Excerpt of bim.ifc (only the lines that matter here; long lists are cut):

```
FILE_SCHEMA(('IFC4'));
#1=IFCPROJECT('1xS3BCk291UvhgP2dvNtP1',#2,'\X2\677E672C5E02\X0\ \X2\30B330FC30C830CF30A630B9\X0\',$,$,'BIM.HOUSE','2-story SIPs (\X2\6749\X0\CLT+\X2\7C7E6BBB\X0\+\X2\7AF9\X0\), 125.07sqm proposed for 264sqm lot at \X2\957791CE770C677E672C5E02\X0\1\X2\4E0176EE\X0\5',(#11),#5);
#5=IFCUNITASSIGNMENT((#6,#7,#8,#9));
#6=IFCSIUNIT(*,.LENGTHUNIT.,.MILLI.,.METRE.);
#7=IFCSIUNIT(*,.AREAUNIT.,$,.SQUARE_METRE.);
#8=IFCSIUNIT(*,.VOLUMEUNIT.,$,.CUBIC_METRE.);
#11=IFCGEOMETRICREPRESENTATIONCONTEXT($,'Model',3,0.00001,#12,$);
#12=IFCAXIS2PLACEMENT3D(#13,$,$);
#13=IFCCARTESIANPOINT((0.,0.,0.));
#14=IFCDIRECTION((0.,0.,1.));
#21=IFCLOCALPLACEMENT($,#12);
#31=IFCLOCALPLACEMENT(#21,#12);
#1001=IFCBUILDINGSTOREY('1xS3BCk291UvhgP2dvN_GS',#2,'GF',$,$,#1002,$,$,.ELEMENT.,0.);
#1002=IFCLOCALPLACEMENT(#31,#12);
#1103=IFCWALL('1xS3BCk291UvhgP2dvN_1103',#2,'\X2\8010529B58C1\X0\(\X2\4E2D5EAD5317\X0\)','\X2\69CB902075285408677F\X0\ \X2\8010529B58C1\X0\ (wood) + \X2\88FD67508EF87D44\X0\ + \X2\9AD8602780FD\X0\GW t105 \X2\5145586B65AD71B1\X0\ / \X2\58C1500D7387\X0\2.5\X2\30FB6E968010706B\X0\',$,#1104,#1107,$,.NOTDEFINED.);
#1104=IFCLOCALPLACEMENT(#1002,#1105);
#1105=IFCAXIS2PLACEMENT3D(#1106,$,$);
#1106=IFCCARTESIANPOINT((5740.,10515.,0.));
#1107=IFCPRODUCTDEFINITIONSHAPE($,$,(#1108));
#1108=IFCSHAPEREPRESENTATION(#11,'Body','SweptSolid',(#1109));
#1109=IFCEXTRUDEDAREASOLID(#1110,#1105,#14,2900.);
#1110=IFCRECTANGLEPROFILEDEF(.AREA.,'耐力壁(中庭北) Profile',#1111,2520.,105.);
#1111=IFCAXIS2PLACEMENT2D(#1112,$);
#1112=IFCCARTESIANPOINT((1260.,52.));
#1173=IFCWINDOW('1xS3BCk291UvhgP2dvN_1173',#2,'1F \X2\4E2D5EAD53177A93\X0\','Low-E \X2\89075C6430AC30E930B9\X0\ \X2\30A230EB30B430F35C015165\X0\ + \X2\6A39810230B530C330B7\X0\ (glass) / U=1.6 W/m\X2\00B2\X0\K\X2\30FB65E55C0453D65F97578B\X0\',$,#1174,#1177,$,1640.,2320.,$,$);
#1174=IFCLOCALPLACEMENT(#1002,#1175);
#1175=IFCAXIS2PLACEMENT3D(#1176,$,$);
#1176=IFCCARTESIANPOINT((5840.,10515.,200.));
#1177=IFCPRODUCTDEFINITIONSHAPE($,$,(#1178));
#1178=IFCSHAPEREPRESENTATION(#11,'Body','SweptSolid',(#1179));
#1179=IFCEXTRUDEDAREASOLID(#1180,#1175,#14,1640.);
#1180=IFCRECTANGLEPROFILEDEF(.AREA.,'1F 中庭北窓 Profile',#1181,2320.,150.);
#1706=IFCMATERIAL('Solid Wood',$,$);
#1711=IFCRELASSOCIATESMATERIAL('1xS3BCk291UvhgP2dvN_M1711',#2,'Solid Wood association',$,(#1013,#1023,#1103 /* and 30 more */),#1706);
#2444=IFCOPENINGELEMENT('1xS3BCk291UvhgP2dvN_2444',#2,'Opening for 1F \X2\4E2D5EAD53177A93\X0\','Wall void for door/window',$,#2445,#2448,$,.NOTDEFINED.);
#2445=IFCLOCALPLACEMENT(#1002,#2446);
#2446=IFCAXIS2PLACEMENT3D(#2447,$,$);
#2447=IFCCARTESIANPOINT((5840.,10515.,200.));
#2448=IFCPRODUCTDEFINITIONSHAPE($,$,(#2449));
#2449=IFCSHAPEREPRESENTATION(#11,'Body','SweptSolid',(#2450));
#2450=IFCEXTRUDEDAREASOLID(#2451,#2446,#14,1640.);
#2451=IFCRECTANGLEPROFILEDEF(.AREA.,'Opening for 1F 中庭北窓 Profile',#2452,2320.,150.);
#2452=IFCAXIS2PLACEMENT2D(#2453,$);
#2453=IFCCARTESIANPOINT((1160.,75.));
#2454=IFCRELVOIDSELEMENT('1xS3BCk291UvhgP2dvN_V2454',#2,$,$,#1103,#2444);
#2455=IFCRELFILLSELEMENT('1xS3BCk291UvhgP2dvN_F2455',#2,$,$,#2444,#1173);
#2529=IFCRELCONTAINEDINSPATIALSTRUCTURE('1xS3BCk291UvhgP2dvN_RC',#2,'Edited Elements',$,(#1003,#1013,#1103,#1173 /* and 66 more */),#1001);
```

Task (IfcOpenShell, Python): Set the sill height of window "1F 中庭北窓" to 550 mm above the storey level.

```python
import numpy as np
import ifcopenshell
import ifcopenshell.api.geometry
import ifcopenshell.geom
import ifcopenshell.util.element
import ifcopenshell.util.placement
import ifcopenshell.util.shape
import ifcopenshell.util.unit

model = ifcopenshell.open("bim.ifc")
unit_scale = ifcopenshell.util.unit.calculate_unit_scale(model)

window = model.by_id(1173)
opening = window.FillsVoids[0].RelatingOpeningElement
storey = ifcopenshell.util.element.get_container(window, ifc_class="IfcBuildingStorey")
level = ifcopenshell.util.placement.get_local_placement(storey.ObjectPlacement)[2, 3]

# The opening's origin need not be at the sill, so measure its lowest point.
shape = ifcopenshell.geom.create_shape(ifcopenshell.geom.settings(), opening)
bottom = ifcopenshell.util.shape.get_shape_bottom_elevation(shape, shape.geometry) / unit_scale
dz = level + 0.55 / unit_scale - bottom

shift = np.array([0.0, 0.0, dz])
# The window is not placed relative to its opening, so move both.
for product in (opening, window):
    matrix = ifcopenshell.util.placement.get_local_placement(product.ObjectPlacement)
    matrix[:3, 3] += shift
    ifcopenshell.api.geometry.edit_object_placement(model, product=product, matrix=matrix, is_si=False)

print(f"moved by {dz * unit_scale:+.3f} m")

model.write("bim_updated.ifc")
```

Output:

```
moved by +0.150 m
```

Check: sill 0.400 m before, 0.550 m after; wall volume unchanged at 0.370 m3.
